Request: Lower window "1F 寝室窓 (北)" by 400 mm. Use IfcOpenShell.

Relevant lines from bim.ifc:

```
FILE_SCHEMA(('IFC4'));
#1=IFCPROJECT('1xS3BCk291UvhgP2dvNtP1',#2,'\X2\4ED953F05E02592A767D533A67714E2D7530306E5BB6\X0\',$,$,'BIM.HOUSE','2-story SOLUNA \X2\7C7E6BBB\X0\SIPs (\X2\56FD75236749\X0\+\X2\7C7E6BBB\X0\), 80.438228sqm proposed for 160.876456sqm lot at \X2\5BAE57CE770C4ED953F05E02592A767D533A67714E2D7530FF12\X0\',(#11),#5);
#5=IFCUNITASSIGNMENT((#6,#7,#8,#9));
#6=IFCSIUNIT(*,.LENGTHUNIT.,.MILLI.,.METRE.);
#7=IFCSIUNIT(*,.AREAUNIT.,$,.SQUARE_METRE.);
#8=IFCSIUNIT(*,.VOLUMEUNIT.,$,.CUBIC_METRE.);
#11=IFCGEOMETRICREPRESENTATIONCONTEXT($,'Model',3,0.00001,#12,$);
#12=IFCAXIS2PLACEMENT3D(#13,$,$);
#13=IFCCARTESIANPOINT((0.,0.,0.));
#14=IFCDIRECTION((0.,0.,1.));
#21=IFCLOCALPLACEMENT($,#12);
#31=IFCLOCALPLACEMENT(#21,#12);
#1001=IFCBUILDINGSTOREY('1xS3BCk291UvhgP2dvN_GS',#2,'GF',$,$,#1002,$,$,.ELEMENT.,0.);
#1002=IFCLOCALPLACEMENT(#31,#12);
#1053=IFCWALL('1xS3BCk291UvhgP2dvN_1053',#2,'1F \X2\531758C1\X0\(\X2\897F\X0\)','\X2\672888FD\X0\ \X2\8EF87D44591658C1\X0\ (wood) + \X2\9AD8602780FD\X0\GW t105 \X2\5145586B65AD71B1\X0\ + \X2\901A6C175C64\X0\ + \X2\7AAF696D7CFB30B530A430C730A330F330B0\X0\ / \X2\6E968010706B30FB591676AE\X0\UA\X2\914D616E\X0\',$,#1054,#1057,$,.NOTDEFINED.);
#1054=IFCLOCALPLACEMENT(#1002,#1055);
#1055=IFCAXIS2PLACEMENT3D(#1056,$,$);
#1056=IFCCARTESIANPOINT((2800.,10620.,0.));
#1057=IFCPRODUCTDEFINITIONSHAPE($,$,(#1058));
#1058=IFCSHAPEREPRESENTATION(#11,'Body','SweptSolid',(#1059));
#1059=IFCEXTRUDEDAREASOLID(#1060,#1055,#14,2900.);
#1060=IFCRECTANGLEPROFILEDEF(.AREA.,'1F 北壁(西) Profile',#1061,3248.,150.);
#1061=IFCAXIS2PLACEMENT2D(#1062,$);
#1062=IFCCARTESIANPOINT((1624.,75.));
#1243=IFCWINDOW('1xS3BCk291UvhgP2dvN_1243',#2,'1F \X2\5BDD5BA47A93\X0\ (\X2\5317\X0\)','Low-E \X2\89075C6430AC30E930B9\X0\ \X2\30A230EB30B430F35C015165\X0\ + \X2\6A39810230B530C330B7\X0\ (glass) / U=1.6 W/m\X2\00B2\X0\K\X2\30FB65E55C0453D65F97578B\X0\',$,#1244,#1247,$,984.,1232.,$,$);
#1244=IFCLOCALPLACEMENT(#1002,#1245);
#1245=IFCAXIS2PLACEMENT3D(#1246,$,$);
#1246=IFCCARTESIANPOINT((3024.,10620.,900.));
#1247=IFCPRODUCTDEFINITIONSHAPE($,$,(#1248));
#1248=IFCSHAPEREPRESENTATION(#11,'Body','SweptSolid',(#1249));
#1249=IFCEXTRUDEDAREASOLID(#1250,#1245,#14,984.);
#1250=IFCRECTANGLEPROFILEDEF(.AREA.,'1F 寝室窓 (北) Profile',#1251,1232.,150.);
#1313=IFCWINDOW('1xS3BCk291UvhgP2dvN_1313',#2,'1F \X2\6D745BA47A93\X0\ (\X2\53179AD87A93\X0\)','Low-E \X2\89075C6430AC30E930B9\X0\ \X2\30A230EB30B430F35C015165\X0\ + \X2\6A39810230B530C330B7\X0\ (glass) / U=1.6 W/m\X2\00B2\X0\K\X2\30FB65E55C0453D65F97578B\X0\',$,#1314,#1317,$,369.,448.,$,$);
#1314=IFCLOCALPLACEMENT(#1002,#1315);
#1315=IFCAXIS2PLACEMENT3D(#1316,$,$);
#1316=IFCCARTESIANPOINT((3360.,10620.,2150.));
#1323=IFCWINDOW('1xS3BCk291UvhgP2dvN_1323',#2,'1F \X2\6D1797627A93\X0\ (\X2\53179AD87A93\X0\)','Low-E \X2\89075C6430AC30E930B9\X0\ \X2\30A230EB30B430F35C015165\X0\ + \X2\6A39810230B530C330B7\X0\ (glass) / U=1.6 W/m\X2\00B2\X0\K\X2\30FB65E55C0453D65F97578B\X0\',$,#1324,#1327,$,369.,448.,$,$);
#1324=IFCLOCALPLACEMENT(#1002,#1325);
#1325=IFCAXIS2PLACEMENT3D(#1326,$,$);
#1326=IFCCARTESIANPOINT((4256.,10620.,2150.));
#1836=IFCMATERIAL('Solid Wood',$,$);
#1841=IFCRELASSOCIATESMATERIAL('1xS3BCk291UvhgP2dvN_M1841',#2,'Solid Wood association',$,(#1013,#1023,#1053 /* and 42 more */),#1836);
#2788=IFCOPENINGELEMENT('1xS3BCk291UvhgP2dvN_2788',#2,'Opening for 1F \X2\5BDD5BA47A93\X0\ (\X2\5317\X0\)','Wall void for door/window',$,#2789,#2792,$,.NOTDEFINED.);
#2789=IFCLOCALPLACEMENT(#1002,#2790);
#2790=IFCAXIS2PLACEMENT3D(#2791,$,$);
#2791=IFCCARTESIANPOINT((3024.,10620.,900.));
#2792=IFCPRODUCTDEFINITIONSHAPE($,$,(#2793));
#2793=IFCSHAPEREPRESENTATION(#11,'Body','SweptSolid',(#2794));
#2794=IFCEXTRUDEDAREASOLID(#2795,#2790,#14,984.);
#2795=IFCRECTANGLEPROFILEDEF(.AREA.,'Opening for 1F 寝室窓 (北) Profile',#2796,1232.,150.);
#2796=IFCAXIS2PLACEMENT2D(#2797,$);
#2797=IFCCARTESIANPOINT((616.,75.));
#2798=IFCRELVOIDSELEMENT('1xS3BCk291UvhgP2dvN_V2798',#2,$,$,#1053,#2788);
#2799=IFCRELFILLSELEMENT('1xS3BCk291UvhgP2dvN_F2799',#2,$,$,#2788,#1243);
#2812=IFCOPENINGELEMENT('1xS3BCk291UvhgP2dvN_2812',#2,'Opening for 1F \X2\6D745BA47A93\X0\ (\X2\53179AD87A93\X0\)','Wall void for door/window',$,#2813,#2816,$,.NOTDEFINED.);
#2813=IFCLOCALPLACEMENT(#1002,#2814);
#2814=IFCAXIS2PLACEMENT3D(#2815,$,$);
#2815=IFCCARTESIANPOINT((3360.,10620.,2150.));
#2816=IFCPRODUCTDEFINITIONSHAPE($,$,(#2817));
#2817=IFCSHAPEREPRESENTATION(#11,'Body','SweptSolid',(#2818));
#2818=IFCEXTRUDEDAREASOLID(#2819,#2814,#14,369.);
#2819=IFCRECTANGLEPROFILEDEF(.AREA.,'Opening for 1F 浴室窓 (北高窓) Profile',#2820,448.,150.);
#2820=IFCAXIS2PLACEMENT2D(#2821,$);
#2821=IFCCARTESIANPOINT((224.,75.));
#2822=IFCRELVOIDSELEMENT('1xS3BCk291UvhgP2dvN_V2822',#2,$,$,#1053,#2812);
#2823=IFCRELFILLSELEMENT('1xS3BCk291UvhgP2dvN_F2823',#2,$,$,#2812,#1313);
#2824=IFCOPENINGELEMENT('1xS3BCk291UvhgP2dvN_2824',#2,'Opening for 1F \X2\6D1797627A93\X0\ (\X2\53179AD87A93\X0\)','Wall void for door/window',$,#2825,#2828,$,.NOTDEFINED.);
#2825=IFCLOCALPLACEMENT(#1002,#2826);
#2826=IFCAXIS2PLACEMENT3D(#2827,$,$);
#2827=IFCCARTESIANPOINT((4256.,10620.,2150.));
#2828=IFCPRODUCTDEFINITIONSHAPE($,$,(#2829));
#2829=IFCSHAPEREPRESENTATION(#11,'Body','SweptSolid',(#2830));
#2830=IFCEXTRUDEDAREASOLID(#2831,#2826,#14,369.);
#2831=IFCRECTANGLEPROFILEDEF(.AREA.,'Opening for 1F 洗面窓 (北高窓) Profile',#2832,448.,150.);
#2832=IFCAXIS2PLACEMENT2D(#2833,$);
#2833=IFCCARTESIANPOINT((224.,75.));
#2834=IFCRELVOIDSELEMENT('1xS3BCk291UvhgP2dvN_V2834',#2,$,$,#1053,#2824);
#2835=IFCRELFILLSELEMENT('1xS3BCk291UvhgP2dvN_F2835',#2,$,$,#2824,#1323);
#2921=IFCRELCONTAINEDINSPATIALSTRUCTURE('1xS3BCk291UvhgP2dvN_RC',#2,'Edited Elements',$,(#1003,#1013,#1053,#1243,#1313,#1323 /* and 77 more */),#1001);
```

```python
import numpy as np
import ifcopenshell
import ifcopenshell.api.geometry
import ifcopenshell.util.placement
import ifcopenshell.util.unit

model = ifcopenshell.open("bim.ifc")
unit_scale = ifcopenshell.util.unit.calculate_unit_scale(model)

window = model.by_guid("1xS3BCk291UvhgP2dvN_1243")
opening = window.FillsVoids[0].RelatingOpeningElement
dz = -0.4 / unit_scale

shift = np.array([0.0, 0.0, dz])
# The window is not placed relative to its opening, so move both.
for product in (opening, window):
    matrix = ifcopenshell.util.placement.get_local_placement(product.ObjectPlacement)
    matrix[:3, 3] += shift
    ifcopenshell.api.geometry.edit_object_placement(model, product=product, matrix=matrix, is_si=False)

print(f"moved by {dz * unit_scale:+.3f} m")

model.write("bim_edited.ifc")
```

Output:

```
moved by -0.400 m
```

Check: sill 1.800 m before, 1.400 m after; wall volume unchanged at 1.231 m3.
